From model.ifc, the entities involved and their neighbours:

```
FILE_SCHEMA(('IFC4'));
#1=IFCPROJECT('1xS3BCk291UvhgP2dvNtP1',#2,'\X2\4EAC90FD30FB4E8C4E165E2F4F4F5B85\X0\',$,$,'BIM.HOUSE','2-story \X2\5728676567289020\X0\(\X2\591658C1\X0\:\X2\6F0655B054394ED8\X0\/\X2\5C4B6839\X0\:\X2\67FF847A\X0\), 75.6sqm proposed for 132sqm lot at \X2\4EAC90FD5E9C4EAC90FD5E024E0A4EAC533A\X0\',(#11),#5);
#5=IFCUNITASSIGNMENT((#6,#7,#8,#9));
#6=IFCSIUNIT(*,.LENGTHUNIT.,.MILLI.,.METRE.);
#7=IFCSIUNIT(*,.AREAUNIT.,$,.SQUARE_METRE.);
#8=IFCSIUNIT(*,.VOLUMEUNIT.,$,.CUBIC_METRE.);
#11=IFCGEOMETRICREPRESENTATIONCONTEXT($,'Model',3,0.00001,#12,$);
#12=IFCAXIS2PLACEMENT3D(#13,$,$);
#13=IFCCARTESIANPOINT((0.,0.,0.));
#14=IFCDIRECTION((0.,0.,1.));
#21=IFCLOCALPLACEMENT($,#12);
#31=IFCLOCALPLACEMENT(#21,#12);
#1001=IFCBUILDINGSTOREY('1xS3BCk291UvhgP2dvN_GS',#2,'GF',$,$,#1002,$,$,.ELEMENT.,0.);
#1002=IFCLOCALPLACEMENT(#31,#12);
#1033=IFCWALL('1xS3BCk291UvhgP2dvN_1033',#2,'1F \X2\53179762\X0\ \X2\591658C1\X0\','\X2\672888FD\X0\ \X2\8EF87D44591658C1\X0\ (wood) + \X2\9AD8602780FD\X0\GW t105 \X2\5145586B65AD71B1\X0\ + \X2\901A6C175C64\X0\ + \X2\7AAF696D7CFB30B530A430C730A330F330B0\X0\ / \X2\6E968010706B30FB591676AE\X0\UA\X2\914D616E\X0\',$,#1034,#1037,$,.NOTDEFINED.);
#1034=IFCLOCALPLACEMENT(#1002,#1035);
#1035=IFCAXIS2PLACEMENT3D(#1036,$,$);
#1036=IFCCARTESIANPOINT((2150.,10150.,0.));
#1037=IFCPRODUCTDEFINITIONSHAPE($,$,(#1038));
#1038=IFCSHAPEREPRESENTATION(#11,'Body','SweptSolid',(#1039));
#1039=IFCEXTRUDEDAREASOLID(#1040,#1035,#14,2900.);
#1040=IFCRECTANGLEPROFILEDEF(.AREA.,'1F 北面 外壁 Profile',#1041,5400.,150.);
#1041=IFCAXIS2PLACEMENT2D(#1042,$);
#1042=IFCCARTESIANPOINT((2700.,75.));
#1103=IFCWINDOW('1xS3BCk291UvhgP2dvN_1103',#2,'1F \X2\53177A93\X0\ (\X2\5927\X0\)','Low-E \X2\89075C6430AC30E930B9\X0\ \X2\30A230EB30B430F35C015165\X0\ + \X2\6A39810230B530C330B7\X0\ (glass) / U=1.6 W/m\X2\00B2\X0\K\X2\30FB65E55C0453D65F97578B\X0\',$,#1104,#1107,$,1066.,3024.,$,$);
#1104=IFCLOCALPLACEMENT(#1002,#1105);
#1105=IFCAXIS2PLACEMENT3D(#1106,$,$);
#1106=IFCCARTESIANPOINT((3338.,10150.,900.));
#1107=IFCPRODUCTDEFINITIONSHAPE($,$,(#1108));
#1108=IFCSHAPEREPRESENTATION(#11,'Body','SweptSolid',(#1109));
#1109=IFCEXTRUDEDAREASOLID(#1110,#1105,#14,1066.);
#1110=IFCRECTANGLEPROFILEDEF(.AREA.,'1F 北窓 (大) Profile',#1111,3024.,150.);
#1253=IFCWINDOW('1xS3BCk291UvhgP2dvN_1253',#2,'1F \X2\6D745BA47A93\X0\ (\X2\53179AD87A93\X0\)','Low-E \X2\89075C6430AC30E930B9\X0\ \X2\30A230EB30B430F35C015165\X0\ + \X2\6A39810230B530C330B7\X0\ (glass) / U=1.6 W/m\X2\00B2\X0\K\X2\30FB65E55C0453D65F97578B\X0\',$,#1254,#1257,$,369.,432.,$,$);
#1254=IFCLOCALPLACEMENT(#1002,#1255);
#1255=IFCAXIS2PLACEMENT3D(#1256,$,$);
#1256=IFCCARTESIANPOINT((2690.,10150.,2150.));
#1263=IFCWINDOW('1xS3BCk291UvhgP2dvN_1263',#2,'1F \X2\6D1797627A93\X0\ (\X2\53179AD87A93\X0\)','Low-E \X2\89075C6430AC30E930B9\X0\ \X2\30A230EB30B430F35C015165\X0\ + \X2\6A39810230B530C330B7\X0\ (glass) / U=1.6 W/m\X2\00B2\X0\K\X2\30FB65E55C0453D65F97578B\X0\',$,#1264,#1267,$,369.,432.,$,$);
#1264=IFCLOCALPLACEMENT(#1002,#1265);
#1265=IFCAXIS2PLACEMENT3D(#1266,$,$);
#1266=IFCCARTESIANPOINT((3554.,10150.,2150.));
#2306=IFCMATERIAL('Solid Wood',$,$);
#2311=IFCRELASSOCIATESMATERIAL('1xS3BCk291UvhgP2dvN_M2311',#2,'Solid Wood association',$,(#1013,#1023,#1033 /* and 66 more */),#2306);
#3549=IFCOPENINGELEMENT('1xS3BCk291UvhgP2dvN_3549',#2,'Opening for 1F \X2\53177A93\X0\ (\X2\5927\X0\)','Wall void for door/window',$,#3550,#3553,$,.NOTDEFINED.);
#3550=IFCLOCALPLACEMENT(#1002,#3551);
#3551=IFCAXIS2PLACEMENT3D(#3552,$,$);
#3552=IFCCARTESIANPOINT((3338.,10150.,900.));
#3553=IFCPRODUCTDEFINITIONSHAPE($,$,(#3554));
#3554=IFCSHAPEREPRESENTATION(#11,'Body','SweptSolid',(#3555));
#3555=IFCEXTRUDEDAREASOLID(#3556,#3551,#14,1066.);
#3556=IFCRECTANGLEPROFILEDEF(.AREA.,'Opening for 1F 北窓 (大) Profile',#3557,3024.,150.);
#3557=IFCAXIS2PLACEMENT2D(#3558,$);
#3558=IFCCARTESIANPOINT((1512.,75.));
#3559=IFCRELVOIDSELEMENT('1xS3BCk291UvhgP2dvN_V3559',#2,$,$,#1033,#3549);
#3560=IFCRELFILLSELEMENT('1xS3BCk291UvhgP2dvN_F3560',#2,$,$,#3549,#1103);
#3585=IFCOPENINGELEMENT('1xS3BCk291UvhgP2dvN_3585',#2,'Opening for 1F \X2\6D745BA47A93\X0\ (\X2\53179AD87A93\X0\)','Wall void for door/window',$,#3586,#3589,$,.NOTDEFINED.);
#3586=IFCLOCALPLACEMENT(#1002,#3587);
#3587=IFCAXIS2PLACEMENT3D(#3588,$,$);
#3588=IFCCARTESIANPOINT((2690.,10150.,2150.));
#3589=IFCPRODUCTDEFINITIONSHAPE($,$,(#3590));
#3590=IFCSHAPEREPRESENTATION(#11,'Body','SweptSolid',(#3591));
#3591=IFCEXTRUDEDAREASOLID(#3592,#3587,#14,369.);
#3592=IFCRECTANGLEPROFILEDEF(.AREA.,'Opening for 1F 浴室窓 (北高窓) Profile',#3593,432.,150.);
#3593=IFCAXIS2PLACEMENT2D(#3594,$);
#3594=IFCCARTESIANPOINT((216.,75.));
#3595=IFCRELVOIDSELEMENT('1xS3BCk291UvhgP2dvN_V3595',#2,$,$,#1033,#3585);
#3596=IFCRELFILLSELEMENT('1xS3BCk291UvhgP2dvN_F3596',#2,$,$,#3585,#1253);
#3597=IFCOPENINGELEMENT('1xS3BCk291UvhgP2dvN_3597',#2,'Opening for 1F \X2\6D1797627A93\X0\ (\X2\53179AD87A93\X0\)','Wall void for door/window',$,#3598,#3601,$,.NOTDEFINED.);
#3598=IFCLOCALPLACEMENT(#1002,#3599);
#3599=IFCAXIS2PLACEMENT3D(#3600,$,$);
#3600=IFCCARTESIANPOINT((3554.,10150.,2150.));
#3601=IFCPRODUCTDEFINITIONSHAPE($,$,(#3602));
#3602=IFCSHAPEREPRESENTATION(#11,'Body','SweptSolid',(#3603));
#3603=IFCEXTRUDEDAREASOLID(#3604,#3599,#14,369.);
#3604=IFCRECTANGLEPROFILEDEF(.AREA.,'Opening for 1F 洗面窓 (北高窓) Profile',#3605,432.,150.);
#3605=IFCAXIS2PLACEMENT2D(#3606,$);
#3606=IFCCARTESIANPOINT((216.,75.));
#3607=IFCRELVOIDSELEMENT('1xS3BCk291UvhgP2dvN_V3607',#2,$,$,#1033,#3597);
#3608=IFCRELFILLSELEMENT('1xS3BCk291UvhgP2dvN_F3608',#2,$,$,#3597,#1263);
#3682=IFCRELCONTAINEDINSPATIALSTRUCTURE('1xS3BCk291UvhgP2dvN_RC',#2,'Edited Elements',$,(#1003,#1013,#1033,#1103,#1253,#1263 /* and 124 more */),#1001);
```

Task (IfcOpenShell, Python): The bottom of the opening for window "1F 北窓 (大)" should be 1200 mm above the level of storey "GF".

```python
import numpy as np
import ifcopenshell
import ifcopenshell.api.geometry
import ifcopenshell.geom
import ifcopenshell.util.element
import ifcopenshell.util.placement
import ifcopenshell.util.shape
import ifcopenshell.util.unit

model = ifcopenshell.open("model.ifc")
unit_scale = ifcopenshell.util.unit.calculate_unit_scale(model)

window = model.by_guid("1xS3BCk291UvhgP2dvN_1103")
opening = window.FillsVoids[0].RelatingOpeningElement
storey = ifcopenshell.util.element.get_container(window, ifc_class="IfcBuildingStorey")
level = ifcopenshell.util.placement.get_local_placement(storey.ObjectPlacement)[2, 3]

# The opening's origin need not be at the sill, so measure its lowest point.
shape = ifcopenshell.geom.create_shape(ifcopenshell.geom.settings(), opening)
bottom = ifcopenshell.util.shape.get_shape_bottom_elevation(shape, shape.geometry) / unit_scale
dz = level + 1.2 / unit_scale - bottom

shift = np.array([0.0, 0.0, dz])
# The window is not placed relative to its opening, so move both.
for product in (opening, window):
    matrix = ifcopenshell.util.placement.get_local_placement(product.ObjectPlacement)
    matrix[:3, 3] += shift
    ifcopenshell.api.geometry.edit_object_placement(model, product=product, matrix=matrix, is_si=False)

print(f"moved by {dz * unit_scale:+.3f} m")

model.write("model-out.ifc")
```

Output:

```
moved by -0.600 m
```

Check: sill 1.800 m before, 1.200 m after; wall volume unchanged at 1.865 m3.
